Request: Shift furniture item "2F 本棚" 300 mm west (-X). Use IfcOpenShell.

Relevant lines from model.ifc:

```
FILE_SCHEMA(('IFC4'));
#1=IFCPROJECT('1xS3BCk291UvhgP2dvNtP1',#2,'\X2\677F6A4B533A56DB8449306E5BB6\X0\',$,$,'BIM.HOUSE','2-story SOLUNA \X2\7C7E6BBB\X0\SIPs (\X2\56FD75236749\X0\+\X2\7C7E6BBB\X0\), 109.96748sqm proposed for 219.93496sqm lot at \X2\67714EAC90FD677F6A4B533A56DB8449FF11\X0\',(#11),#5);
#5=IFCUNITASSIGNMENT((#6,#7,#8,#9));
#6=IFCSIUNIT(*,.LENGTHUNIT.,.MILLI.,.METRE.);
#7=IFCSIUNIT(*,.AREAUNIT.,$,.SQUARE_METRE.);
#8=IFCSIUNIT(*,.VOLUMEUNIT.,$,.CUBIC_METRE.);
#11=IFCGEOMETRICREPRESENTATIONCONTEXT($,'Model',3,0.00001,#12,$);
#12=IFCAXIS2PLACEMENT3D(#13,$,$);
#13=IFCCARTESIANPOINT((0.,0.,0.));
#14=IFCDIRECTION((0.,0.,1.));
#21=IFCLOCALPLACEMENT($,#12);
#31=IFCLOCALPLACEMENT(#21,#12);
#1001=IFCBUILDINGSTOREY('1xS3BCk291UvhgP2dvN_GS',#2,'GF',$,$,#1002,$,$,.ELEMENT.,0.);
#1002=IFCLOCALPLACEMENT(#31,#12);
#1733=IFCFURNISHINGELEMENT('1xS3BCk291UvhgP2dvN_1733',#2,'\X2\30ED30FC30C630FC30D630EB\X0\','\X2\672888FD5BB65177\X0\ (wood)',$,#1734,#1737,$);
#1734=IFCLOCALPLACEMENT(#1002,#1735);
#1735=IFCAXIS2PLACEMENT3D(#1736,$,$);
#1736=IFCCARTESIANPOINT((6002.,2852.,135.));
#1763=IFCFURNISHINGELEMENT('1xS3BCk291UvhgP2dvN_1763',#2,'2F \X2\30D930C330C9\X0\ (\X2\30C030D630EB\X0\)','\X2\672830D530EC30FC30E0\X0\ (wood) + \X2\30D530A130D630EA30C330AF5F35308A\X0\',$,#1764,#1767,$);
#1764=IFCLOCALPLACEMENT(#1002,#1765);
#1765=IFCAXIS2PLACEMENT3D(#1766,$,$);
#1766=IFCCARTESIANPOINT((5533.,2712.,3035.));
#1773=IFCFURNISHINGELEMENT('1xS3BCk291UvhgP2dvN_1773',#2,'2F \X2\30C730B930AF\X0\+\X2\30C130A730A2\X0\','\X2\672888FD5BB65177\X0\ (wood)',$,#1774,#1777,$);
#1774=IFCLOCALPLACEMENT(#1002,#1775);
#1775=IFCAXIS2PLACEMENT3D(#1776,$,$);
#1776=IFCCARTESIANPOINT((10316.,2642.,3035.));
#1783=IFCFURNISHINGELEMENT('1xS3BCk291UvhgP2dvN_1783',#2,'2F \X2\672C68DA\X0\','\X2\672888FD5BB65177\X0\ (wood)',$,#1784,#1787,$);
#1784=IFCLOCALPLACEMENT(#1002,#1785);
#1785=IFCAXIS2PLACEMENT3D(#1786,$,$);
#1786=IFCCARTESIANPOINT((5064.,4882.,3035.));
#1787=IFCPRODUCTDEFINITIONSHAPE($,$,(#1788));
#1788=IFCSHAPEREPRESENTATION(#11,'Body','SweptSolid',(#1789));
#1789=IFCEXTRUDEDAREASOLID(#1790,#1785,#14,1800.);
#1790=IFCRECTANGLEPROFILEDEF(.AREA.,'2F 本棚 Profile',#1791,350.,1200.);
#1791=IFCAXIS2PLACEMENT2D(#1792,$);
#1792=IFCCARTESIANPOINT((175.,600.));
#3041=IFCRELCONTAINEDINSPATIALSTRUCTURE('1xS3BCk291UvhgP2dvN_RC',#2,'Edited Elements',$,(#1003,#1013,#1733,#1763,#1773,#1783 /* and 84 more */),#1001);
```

```python
import ifcopenshell
import ifcopenshell.api.geometry
import ifcopenshell.util.placement
import ifcopenshell.util.unit

model = ifcopenshell.open("model.ifc")
unit_scale = ifcopenshell.util.unit.calculate_unit_scale(model)

item = model.by_guid("1xS3BCk291UvhgP2dvN_1783")
matrix = ifcopenshell.util.placement.get_local_placement(item.ObjectPlacement)
matrix[0, 3] -= 0.3 / unit_scale
ifcopenshell.api.geometry.edit_object_placement(model, product=item, matrix=matrix, is_si=False)

print(ifcopenshell.util.placement.get_local_placement(item.ObjectPlacement).round(3) + 0.0)

model.write("model_v2.ifc")
```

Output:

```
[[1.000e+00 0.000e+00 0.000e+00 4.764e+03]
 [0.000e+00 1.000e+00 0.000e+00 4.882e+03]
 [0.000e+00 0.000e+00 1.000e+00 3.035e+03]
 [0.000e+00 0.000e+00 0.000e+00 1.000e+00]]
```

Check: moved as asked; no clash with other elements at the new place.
